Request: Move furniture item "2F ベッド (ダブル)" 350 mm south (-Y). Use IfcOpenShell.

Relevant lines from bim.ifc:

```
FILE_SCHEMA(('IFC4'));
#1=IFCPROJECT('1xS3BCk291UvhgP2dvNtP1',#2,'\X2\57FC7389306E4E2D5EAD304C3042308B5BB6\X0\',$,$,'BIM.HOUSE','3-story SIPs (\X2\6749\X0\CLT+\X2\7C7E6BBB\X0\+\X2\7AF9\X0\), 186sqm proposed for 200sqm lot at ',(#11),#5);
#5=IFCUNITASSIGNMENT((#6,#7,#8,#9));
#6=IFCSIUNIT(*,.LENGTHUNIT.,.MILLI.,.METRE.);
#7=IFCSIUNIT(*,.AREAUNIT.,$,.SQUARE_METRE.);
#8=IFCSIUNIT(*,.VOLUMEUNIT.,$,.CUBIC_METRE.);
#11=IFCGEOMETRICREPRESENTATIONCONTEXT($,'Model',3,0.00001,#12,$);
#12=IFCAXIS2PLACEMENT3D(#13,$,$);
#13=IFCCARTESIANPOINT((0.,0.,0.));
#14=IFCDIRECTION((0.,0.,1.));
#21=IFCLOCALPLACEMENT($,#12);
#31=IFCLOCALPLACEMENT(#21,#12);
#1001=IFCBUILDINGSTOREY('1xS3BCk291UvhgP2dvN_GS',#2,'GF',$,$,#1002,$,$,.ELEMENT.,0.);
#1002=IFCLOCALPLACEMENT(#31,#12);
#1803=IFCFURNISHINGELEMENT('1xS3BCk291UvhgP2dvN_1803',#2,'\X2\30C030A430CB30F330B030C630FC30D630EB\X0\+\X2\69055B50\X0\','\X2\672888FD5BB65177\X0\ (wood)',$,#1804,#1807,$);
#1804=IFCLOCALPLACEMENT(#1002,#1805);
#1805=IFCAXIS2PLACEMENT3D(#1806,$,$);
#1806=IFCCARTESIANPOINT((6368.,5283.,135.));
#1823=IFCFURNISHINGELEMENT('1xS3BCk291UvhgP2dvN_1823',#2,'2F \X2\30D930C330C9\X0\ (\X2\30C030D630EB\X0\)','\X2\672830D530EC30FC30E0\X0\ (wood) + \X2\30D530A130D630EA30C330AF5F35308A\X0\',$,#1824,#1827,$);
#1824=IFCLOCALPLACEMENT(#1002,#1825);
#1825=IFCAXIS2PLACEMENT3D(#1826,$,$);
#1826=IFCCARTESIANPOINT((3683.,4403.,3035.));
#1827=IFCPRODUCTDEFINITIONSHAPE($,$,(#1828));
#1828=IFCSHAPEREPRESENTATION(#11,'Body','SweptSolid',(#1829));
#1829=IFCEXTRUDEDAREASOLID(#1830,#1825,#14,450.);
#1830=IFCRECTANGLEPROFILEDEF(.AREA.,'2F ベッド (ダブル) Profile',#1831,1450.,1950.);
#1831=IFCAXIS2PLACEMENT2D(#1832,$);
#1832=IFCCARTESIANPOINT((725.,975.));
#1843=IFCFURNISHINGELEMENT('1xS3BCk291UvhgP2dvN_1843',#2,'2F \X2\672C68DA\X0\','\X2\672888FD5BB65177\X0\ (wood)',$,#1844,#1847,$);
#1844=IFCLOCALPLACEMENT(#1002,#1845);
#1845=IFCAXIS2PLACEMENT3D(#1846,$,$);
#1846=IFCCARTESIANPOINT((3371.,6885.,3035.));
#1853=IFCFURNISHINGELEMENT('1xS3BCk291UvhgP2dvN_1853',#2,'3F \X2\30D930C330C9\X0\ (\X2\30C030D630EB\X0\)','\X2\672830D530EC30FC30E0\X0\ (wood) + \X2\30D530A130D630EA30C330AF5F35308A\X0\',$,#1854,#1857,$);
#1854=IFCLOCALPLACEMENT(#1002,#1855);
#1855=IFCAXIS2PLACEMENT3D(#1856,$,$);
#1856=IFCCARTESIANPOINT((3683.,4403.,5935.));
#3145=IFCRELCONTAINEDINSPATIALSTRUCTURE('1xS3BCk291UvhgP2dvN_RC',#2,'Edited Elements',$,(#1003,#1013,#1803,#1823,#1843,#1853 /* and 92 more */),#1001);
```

```python
import ifcopenshell
import ifcopenshell.api.geometry
import ifcopenshell.util.placement

model = ifcopenshell.open("bim.ifc")

item = model.by_id(1823)
matrix = ifcopenshell.util.placement.get_local_placement(item.ObjectPlacement)
matrix[1, 3] -= 350.0
ifcopenshell.api.geometry.edit_object_placement(model, product=item, matrix=matrix, is_si=False)

print(ifcopenshell.util.placement.get_local_placement(item.ObjectPlacement).round(3) + 0.0)

model.write("bim-out.ifc")
```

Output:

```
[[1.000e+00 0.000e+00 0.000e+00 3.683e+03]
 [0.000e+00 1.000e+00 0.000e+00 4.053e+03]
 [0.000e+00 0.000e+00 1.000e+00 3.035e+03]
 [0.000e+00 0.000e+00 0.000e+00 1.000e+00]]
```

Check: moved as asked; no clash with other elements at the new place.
